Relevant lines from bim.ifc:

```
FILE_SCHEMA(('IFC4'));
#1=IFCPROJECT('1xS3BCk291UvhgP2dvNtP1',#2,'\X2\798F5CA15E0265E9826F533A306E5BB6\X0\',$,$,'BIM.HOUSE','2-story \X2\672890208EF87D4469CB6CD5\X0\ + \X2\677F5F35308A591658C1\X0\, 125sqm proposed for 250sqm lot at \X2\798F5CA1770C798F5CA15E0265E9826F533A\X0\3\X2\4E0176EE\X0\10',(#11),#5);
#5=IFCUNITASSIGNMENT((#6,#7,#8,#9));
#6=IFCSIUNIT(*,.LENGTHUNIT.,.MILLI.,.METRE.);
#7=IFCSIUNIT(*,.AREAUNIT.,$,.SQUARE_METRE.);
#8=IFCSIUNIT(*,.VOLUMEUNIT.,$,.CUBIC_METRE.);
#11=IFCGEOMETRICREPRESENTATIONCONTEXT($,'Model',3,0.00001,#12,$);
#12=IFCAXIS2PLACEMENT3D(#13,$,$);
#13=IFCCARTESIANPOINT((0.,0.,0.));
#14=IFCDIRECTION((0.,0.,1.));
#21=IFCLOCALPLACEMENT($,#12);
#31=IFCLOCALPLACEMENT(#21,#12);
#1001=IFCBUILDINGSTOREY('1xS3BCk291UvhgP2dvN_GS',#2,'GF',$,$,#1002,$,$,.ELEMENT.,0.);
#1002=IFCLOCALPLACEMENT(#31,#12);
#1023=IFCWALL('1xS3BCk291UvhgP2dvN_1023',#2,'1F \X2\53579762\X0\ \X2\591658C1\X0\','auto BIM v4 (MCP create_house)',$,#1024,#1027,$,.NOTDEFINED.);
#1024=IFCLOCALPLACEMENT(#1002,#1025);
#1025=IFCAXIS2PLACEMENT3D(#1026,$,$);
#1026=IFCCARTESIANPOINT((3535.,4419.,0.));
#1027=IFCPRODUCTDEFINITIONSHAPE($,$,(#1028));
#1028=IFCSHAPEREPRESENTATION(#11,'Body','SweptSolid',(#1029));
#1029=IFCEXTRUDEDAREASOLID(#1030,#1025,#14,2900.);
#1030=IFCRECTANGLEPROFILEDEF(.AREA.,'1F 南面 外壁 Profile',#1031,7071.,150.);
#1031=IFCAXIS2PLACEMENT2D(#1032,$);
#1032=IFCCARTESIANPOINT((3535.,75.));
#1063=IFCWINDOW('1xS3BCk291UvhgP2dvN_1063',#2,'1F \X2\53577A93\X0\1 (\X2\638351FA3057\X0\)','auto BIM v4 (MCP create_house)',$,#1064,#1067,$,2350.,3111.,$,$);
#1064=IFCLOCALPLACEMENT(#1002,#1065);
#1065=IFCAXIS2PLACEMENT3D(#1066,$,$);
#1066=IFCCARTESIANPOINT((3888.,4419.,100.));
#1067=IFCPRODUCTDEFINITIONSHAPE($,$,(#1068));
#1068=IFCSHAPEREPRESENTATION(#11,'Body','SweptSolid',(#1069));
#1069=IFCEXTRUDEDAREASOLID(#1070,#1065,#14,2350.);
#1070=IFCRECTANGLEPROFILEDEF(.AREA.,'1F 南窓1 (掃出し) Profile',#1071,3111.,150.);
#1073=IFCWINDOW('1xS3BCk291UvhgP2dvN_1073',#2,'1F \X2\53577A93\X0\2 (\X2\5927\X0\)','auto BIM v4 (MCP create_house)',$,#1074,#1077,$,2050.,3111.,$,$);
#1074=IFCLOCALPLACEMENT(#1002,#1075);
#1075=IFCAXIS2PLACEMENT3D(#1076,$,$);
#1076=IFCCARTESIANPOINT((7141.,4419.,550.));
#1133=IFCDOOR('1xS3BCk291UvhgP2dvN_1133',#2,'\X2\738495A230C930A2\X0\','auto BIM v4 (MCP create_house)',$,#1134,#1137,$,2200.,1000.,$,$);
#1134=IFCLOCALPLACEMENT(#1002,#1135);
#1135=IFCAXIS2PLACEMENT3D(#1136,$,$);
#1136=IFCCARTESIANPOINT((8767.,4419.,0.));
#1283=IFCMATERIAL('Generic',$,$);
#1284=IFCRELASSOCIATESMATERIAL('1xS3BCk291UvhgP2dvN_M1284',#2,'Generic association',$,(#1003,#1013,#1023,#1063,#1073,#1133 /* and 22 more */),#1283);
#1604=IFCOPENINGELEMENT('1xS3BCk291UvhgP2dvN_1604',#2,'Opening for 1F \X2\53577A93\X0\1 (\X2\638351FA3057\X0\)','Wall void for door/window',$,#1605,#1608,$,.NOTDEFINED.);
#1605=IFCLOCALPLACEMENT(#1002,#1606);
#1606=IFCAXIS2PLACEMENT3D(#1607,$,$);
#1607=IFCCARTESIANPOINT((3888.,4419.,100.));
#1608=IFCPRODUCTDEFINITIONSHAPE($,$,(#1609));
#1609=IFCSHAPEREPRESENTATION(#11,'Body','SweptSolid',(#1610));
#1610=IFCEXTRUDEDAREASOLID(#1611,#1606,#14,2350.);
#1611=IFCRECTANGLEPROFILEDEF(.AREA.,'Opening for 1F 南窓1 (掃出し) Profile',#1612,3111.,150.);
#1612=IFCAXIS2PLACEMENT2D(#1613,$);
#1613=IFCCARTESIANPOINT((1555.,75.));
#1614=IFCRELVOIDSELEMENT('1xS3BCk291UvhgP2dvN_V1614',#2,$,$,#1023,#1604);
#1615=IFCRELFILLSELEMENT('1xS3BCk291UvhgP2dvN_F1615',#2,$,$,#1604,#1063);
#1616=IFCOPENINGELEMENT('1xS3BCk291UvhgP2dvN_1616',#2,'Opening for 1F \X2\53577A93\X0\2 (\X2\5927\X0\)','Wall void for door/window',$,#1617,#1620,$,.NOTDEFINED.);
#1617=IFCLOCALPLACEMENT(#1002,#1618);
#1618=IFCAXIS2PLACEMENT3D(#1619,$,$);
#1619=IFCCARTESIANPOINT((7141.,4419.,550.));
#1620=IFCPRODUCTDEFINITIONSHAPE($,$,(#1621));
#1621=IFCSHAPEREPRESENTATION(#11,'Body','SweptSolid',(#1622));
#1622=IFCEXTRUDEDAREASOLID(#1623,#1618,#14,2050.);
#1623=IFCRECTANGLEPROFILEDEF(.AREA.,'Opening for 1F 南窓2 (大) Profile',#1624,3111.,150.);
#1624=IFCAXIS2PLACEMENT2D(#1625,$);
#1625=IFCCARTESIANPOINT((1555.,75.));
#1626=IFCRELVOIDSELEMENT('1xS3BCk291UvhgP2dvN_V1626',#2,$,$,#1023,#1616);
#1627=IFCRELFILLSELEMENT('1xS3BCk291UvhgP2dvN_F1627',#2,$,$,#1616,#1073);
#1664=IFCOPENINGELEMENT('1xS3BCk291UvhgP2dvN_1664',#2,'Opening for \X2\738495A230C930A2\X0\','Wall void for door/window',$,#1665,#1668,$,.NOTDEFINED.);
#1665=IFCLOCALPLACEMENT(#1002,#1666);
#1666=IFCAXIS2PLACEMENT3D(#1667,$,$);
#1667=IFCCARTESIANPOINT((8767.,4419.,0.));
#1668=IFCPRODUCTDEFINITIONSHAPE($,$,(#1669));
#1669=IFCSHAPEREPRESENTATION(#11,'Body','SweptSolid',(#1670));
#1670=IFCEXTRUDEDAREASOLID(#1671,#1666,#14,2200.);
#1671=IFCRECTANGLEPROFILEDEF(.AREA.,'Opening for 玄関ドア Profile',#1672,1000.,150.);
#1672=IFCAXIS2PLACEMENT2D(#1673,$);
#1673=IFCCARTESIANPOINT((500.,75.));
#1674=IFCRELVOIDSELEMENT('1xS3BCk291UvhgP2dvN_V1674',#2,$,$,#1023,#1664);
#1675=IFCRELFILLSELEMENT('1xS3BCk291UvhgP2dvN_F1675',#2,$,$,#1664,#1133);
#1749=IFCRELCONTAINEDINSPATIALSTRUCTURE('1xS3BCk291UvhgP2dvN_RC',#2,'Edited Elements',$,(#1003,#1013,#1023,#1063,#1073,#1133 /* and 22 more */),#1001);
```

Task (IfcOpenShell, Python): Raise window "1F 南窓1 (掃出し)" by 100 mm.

```python
import numpy as np
import ifcopenshell
import ifcopenshell.api.geometry
import ifcopenshell.util.placement
import ifcopenshell.util.unit

model = ifcopenshell.open("bim.ifc")
unit_scale = ifcopenshell.util.unit.calculate_unit_scale(model)

window = model.by_id(1063)
opening = window.FillsVoids[0].RelatingOpeningElement
dz = 0.1 / unit_scale

shift = np.array([0.0, 0.0, dz])
# The window is not placed relative to its opening, so move both.
for product in (opening, window):
    matrix = ifcopenshell.util.placement.get_local_placement(product.ObjectPlacement)
    matrix[:3, 3] += shift
    ifcopenshell.api.geometry.edit_object_placement(model, product=product, matrix=matrix, is_si=False)

print(f"moved by {dz * unit_scale:+.3f} m")

model.write("bim_updated.ifc")
```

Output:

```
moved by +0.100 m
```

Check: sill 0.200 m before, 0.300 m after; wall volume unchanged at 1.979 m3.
